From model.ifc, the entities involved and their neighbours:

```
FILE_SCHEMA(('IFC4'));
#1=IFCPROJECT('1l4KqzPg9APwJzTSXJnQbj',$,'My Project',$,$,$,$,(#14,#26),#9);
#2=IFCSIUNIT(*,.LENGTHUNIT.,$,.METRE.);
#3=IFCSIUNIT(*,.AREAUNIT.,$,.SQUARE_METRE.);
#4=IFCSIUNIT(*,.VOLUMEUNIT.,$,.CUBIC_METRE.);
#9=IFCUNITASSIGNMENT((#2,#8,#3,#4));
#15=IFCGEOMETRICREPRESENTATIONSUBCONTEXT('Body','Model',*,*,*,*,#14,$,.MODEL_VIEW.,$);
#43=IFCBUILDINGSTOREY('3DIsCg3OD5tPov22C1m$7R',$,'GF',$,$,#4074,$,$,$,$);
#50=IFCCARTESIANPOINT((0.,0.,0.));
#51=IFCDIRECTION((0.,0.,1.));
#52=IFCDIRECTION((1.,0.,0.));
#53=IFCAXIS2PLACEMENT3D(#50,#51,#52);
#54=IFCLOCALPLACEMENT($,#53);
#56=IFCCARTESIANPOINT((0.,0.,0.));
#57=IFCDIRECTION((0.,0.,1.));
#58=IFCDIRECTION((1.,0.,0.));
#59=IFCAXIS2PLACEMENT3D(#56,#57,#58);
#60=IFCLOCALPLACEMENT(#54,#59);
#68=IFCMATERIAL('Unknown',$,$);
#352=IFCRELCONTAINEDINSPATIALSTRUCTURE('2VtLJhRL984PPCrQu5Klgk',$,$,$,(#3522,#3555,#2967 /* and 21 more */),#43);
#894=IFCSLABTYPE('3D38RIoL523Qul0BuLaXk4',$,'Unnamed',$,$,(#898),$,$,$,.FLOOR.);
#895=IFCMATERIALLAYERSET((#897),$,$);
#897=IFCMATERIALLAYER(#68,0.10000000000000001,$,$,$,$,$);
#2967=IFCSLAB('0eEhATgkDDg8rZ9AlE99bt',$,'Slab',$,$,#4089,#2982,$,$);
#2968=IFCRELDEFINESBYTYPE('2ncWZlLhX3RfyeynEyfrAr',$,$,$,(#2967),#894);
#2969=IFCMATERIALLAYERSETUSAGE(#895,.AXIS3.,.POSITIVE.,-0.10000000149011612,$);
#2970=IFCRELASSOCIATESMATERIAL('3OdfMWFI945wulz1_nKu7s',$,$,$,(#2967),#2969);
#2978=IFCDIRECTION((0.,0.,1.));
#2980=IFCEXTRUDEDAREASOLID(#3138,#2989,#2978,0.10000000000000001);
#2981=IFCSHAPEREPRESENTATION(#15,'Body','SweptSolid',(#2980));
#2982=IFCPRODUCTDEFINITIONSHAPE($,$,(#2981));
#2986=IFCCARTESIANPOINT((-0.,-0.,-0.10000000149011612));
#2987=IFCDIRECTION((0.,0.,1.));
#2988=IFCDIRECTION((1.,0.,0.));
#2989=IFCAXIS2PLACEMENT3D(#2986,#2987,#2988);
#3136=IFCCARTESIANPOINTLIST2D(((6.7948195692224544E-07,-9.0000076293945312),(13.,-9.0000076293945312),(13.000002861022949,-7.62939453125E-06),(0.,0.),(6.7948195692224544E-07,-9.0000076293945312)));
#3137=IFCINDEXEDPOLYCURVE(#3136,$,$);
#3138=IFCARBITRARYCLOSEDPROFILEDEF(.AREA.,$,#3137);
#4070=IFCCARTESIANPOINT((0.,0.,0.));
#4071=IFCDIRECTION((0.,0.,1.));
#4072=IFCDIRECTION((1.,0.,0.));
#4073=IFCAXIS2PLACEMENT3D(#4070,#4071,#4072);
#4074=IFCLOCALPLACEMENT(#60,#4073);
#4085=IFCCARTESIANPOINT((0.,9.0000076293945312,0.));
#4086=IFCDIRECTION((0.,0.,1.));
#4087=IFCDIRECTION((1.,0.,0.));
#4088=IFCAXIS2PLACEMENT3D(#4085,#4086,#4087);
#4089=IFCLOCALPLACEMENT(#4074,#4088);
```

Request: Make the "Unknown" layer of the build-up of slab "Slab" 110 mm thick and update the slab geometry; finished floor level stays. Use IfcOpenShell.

```python
import ifcopenshell
import ifcopenshell.util.element
import ifcopenshell.util.representation
import ifcopenshell.util.unit

model = ifcopenshell.open("model.ifc")
unit_scale = ifcopenshell.util.unit.calculate_unit_scale(model)

layer_set = model.by_id(895)
layer = next(l for l in layer_set.MaterialLayers if l.Material and l.Material.Name == "Unknown")
change = 0.11 / unit_scale - layer.LayerThickness
layer.LayerThickness += change

# Geometry does not follow the layer set by itself.
slabs = [e for e in ifcopenshell.util.element.get_elements_by_material(model, layer_set) if e.is_a("IfcSlab")]
for slab in sorted(slabs, key=lambda e: e.id()):
    body = ifcopenshell.util.representation.get_representation(slab, "Model", "Body")
    solid = body.Items[0]
    old_depth = solid.Depth
    solid.Depth += change
    # Extruded upwards: lower the start of the extrusion so the top stays.
    x, y, z = solid.Position.Location.Coordinates
    solid.Position.Location = model.createIfcCartesianPoint((x, y, z - change))
    print(slab.id(), f"{old_depth:g} -> {solid.Depth:g}")

# The layers are counted up from the underside, which has moved.
for usage in {ifcopenshell.util.element.get_material(slab) for slab in slabs}:
    usage.OffsetFromReferenceLine -= change

model.write("model_updated.ifc")
```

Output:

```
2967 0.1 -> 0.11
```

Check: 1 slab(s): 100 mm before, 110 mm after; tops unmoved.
